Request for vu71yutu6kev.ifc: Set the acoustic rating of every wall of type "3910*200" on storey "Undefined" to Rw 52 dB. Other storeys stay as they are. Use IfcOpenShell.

First a look at what the model holds.

```python
import ifcopenshell
import ifcopenshell.util.element

model = ifcopenshell.open("vu71yutu6kev.ifc")
print(model.schema)
storey = next(s for s in model.by_type("IfcBuildingStorey") if s.Name == "Undefined")
walls = [e for e in ifcopenshell.util.element.get_decomposition(storey) if e.is_a("IfcWall")]
seen = {}
for e in walls:
    element_type = ifcopenshell.util.element.get_type(e)
    key = (element_type.Name if element_type != e and element_type else None, ifcopenshell.util.element.get_pset(e, "Pset_WallCommon", "AcousticRating"))
    seen[key] = seen.get(key, 0) + 1
for (name, value), count in sorted(seen.items(), key=str):
    print(count, "x", name, "|", value)
```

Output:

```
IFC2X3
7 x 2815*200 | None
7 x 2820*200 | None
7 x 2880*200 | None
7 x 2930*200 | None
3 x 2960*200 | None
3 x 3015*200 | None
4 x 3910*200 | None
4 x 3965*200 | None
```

```python
import ifcopenshell
import ifcopenshell.api.pset
import ifcopenshell.util.element

model = ifcopenshell.open("vu71yutu6kev.ifc")

storey = next(s for s in model.by_type("IfcBuildingStorey") if s.Name == "Undefined")
walls = [e for e in ifcopenshell.util.element.get_decomposition(storey) if e.is_a("IfcWall")]

count = 0
for e in walls:
    element_type = ifcopenshell.util.element.get_type(e)
    if element_type in (None, e) or element_type.Name != "3910*200":
        continue
    # add_pset returns the element's existing set when there is one.
    pset = ifcopenshell.api.pset.add_pset(model, product=e, name="Pset_WallCommon")
    ifcopenshell.api.pset.edit_pset(model, pset=pset, properties={"AcousticRating": "Rw 52 dB"})
    count += 1

print(count, "walls updated")

model.write("vu71yutu6kev_v2.ifc")
```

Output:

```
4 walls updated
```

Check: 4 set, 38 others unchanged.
